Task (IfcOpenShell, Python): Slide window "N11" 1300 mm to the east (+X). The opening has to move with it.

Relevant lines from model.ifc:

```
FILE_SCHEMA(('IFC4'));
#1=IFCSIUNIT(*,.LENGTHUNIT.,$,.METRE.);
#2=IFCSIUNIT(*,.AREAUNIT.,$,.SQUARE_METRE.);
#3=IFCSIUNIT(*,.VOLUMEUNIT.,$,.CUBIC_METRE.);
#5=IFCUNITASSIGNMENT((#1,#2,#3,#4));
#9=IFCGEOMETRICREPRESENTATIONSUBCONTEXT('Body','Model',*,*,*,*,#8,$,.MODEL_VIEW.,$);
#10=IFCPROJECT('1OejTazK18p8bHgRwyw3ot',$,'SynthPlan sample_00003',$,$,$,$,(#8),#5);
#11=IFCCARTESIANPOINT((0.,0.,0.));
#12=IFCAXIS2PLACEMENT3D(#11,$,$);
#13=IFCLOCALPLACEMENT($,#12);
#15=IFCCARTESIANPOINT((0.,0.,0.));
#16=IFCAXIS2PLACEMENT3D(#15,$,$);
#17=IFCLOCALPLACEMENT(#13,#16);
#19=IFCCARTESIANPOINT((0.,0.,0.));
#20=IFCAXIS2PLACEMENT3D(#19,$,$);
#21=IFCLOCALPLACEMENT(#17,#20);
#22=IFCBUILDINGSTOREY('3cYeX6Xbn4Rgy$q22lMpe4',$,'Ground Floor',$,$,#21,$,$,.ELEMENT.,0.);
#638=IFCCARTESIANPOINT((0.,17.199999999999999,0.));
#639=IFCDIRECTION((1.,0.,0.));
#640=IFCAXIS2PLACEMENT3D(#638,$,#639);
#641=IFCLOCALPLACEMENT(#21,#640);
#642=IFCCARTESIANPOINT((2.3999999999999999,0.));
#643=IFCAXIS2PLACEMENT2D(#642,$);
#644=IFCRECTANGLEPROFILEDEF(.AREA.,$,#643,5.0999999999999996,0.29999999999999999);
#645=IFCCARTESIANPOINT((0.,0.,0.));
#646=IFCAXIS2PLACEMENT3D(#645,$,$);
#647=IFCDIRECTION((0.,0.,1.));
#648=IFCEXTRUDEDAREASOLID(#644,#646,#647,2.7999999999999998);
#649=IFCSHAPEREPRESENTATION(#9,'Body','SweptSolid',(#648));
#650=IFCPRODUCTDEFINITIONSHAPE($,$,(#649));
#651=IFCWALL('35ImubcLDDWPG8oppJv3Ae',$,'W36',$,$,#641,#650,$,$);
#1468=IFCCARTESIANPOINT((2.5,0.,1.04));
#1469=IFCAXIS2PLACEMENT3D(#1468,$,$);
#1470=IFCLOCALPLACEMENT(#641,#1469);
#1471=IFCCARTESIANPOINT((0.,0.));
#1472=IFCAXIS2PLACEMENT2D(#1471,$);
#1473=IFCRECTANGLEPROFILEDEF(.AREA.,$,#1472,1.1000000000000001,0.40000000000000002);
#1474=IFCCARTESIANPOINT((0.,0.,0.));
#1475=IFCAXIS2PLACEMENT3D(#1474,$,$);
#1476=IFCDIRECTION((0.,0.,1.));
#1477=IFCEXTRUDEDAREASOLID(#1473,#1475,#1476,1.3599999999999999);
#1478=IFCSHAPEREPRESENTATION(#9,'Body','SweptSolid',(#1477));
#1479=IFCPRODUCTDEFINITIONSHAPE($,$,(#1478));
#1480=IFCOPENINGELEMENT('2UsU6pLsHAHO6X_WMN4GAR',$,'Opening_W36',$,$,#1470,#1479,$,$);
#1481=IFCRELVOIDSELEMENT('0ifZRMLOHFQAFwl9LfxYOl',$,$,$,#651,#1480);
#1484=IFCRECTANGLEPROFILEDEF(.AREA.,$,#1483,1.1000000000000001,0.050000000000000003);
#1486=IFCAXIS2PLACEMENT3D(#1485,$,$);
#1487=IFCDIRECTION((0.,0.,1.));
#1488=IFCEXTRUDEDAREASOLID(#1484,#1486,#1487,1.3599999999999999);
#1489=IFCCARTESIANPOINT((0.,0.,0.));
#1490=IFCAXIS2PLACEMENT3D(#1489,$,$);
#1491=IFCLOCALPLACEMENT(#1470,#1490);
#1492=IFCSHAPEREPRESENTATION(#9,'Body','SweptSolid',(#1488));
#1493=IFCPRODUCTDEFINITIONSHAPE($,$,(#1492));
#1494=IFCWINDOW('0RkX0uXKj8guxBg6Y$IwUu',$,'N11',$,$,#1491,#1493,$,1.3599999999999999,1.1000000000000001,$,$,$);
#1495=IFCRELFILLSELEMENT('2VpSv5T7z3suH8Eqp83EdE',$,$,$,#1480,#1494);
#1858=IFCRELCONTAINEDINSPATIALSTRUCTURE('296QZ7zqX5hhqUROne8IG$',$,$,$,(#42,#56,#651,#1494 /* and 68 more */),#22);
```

```python
import ifcopenshell
import ifcopenshell.api.geometry
import ifcopenshell.util.placement

model = ifcopenshell.open("model.ifc")

window = model.by_guid("0RkX0uXKj8guxBg6Y$IwUu")
opening = window.FillsVoids[0].RelatingOpeningElement
wall = opening.VoidsElements[0].RelatingBuildingElement

wall_matrix = ifcopenshell.util.placement.get_local_placement(wall.ObjectPlacement)
shift = wall_matrix[:3, 0] * 1.3
before = ifcopenshell.util.placement.get_local_placement(window.ObjectPlacement)[:3, 3].copy()

# The window is placed relative to its opening, so it follows when the opening moves.
matrix = ifcopenshell.util.placement.get_local_placement(opening.ObjectPlacement)
matrix[:3, 3] += shift
ifcopenshell.api.geometry.edit_object_placement(
    model, product=opening, matrix=matrix, is_si=False, should_transform_children=True
)

after = ifcopenshell.util.placement.get_local_placement(window.ObjectPlacement)[:3, 3]
print("window moved by", (after - before).round(3) + 0.0)

model.write("model_rev.ifc")
```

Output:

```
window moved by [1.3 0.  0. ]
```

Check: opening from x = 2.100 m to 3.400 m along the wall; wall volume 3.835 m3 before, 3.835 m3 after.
